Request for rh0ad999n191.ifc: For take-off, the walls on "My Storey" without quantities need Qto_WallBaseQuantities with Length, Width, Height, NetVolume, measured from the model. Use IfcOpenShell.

First a look at what the model holds.

```python
import ifcopenshell
import ifcopenshell.util.element
import ifcopenshell.util.unit

model = ifcopenshell.open("rh0ad999n191.ifc")
print(model.schema)
for unit_type in ("LENGTHUNIT", "AREAUNIT", "VOLUMEUNIT"):
    print(unit_type, ifcopenshell.util.unit.calculate_unit_scale(model, unit_type))
storey = next(s for s in model.by_type("IfcBuildingStorey") if s.Name == "My Storey")
walls = [e for e in ifcopenshell.util.element.get_decomposition(storey) if e.is_a("IfcWall")]
for e in sorted(walls, key=lambda e: e.id()):
    print(e.id(), e.is_a(), e.Name, list(ifcopenshell.util.element.get_psets(e, qtos_only=True)), sep=" | ")
```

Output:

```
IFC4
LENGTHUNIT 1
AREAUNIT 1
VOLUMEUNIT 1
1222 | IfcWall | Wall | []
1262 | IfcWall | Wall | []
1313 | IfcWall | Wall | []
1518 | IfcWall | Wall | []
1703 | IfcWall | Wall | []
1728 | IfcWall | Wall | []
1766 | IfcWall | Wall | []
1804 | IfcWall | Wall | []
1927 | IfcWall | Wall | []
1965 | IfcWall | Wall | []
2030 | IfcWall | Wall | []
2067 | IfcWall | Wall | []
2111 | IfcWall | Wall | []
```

```python
import ifcopenshell
import ifcopenshell.api.pset
import ifcopenshell.geom
import ifcopenshell.util.element
import ifcopenshell.util.shape
import ifcopenshell.util.unit

model = ifcopenshell.open("rh0ad999n191.ifc")
unit_scale = ifcopenshell.util.unit.calculate_unit_scale(model)
volume_scale = ifcopenshell.util.unit.calculate_unit_scale(model, "VOLUMEUNIT")
settings = ifcopenshell.geom.settings()

storey = next(s for s in model.by_type("IfcBuildingStorey") if s.Name == "My Storey")
walls = [e for e in ifcopenshell.util.element.get_decomposition(storey) if e.is_a("IfcWall")]

for e in sorted(walls, key=lambda e: e.id()):
    if ifcopenshell.util.element.get_psets(e, qtos_only=True, should_inherit=False):
        continue
    # Geometry comes back in metres, in the element's own axes.
    shape = ifcopenshell.geom.create_shape(settings, e)
    values = {
        "Length": ifcopenshell.util.shape.get_x(shape.geometry) / unit_scale,
        "Width": ifcopenshell.util.shape.get_y(shape.geometry) / unit_scale,
        "Height": ifcopenshell.util.shape.get_z(shape.geometry) / unit_scale,
        "NetVolume": ifcopenshell.util.shape.get_volume(shape.geometry) / volume_scale,
    }
    qto = ifcopenshell.api.pset.add_qto(model, product=e, name="Qto_WallBaseQuantities")
    ifcopenshell.api.pset.edit_qto(model, qto=qto, properties=values)
    print(e.id(), {k: round(v, 3) for k, v in values.items()})

model.write("rh0ad999n191_edited.ifc")
```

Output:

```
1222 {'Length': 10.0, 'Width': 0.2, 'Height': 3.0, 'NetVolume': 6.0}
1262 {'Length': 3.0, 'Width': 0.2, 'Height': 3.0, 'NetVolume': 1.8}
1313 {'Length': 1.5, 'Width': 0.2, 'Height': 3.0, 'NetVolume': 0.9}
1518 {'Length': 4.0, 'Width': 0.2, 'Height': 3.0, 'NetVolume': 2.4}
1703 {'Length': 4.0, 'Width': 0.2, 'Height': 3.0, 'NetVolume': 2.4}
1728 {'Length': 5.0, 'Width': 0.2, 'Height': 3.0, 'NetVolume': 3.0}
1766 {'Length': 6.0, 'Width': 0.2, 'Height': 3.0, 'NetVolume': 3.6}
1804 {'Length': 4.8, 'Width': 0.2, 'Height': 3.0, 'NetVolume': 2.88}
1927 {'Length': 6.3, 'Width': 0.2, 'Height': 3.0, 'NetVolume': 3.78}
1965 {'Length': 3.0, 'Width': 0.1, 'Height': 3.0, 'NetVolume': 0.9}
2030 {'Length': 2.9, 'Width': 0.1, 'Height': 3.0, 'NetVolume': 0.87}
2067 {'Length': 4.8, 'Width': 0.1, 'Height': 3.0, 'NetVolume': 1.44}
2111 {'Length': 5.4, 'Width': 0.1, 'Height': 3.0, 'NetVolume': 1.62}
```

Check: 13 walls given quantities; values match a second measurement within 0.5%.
